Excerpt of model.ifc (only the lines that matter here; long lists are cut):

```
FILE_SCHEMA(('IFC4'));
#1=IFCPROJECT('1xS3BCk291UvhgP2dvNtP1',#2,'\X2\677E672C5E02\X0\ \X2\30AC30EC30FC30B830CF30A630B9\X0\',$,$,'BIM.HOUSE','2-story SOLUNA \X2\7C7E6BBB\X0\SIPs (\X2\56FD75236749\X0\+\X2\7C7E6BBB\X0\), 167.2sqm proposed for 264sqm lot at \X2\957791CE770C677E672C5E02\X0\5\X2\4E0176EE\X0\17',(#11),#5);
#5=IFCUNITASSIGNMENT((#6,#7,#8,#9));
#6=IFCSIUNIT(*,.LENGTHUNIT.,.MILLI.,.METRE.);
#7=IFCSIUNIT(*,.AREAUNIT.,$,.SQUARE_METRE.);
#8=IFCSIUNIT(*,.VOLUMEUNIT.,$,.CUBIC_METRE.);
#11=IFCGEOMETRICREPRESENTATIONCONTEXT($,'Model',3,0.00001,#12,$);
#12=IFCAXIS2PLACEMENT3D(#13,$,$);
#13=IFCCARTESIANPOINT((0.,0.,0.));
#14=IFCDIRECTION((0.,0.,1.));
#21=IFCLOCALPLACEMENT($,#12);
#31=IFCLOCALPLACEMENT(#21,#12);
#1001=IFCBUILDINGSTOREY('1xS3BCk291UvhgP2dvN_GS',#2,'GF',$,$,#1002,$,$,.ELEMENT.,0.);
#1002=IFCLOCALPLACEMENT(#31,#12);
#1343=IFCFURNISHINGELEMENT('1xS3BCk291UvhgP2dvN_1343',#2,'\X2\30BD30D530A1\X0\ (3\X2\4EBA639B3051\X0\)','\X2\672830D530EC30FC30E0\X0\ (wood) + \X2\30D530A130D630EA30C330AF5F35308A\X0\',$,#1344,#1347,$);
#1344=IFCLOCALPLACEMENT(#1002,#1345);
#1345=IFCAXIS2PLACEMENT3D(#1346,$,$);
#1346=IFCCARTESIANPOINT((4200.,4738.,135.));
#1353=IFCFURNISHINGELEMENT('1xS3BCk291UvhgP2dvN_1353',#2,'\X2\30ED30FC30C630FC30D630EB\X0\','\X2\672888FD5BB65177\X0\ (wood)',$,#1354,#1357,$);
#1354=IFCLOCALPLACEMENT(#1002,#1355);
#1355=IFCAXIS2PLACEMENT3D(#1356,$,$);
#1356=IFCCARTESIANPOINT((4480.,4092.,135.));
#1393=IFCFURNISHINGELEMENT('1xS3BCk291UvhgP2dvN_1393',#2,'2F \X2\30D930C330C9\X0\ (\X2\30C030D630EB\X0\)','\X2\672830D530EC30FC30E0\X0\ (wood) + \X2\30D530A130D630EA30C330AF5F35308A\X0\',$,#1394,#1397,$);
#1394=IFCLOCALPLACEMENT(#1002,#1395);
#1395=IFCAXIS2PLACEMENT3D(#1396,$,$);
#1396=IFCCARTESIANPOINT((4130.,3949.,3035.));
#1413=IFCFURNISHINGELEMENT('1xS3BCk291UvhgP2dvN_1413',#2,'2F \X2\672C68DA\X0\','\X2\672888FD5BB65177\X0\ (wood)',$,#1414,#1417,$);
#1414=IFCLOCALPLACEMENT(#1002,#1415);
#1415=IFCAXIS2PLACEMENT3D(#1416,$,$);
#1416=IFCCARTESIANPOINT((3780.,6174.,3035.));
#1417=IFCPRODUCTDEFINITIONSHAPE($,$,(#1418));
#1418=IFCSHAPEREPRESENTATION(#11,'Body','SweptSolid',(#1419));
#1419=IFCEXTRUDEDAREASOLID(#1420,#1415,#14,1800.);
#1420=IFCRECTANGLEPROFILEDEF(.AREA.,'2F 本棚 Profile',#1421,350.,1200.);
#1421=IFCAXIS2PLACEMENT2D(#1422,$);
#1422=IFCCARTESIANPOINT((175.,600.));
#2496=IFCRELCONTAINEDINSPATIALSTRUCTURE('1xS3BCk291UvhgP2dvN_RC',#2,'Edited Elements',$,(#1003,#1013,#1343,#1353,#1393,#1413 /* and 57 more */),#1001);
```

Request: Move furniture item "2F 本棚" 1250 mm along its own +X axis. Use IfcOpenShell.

```python
import ifcopenshell
import ifcopenshell.api.geometry
import ifcopenshell.util.placement
import ifcopenshell.util.unit

model = ifcopenshell.open("model.ifc")
unit_scale = ifcopenshell.util.unit.calculate_unit_scale(model)

item = model.by_guid("1xS3BCk291UvhgP2dvN_1413")
matrix = ifcopenshell.util.placement.get_local_placement(item.ObjectPlacement)
matrix[:3, 3] += matrix[:3, 0] * 1.25 / unit_scale
ifcopenshell.api.geometry.edit_object_placement(model, product=item, matrix=matrix, is_si=False)

print(ifcopenshell.util.placement.get_local_placement(item.ObjectPlacement).round(3) + 0.0)

model.write("model_edited.ifc")
```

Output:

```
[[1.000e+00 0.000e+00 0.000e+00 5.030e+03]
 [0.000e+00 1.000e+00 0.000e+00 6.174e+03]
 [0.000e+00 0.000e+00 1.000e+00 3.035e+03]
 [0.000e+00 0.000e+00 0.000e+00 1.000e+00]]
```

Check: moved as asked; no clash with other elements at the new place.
